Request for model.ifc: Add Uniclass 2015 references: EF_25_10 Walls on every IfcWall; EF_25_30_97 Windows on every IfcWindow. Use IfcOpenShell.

First a look at what the model holds.

```python
import ifcopenshell

model = ifcopenshell.open("model.ifc")
print(model.schema)
print("classifications:", [c.Name for c in model.by_type("IfcClassification")])
for ifc_class in ("IfcDoor", "IfcRoof", "IfcStair", "IfcWall", "IfcWindow"):
    print(ifc_class, len(model.by_type(ifc_class)))
```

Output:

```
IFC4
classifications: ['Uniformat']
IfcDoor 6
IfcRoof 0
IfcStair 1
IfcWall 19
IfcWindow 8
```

```python
import ifcopenshell
import ifcopenshell.api.classification

model = ifcopenshell.open("model.ifc")

system = ifcopenshell.api.classification.add_classification(model, classification="Uniclass 2015")

codes = {
    "IfcWall": ("EF_25_10", "Walls"),
    "IfcWindow": ("EF_25_30_97", "Windows"),
}
for ifc_class, (code, name) in codes.items():
    products = model.by_type(ifc_class)
    ifcopenshell.api.classification.add_reference(
        model, products=products, classification=system, identification=code, name=name
    )
    print(code, len(products))

model.write("model_updated.ifc")
```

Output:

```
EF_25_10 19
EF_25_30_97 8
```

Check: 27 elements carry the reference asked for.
